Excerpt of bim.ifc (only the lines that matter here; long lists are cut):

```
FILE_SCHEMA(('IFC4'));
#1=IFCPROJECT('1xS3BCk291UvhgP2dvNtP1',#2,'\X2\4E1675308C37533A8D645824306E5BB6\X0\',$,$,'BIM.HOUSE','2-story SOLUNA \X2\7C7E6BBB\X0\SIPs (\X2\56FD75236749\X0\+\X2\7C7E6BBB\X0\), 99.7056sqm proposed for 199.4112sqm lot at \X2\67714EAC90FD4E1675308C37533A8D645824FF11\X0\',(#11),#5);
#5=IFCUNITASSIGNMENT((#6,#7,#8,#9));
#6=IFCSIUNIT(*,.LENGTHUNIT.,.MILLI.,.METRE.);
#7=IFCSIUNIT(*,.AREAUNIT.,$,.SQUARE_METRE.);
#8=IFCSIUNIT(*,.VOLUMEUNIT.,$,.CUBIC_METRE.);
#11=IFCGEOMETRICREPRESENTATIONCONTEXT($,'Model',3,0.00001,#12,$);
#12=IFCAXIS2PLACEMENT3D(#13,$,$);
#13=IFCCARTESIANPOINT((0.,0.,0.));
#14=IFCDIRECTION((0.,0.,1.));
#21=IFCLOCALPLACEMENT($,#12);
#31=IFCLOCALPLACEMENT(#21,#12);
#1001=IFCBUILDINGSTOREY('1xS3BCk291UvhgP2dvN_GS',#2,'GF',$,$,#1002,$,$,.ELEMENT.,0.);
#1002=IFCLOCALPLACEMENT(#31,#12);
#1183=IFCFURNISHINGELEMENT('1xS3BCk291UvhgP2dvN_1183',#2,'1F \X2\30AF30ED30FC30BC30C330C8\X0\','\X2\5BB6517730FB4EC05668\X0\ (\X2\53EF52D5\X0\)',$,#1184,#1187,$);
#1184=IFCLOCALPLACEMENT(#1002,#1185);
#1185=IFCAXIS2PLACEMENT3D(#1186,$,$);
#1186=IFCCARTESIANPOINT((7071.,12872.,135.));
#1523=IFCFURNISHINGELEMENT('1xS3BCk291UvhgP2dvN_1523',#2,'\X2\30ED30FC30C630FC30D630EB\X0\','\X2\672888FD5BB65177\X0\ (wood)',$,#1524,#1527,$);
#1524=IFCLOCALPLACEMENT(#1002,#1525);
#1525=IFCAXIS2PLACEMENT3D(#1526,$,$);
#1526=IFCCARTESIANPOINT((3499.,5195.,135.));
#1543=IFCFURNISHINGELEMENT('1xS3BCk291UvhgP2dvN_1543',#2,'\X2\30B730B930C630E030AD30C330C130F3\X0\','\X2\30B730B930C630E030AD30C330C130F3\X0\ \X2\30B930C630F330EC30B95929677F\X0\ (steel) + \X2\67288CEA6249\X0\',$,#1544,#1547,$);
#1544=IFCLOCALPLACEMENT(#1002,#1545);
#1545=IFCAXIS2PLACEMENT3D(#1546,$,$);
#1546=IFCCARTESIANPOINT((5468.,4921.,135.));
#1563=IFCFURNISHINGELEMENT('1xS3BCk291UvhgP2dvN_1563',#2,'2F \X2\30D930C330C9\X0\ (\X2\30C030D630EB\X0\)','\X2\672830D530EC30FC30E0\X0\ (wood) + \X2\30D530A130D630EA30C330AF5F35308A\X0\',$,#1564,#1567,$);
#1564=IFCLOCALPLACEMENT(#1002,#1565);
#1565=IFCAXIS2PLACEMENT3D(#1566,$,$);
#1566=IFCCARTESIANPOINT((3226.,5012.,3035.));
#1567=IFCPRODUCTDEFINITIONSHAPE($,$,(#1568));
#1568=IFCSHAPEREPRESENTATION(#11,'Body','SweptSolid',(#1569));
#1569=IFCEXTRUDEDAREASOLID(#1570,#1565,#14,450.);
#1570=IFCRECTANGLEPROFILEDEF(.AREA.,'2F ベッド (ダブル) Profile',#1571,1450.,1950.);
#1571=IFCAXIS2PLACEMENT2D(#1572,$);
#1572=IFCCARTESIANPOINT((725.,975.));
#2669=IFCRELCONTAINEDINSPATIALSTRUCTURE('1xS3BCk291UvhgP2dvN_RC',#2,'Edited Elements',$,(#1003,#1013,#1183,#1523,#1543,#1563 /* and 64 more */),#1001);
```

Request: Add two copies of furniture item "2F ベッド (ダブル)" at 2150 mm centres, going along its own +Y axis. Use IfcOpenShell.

```python
import ifcopenshell
import ifcopenshell.api.geometry
import ifcopenshell.api.root
import ifcopenshell.util.element
import ifcopenshell.util.placement
import ifcopenshell.util.unit

model = ifcopenshell.open("bim.ifc")
unit_scale = ifcopenshell.util.unit.calculate_unit_scale(model)


def reuse_history(source, copy):
    """copy_class also copies each property set's owner history, people and application; keep the originals."""
    for rel in copy.IsDefinedBy:
        if rel.is_a("IfcRelDefinesByProperties") and (history := rel.RelatingPropertyDefinition.OwnerHistory):
            rel.RelatingPropertyDefinition.OwnerHistory = source.OwnerHistory
            ifcopenshell.util.element.remove_deep2(model, history)


source = model.by_id(1563)
base = ifcopenshell.util.placement.get_local_placement(source.ObjectPlacement)
step = base[:3, 1] * 2.15 / unit_scale

for i in range(1, 3):
    copy = ifcopenshell.api.root.copy_class(model, product=source)
    copy.Representation = ifcopenshell.util.element.copy_deep(
        model, source.Representation, exclude=["IfcGeometricRepresentationContext", "IfcRepresentationMap"]
    )
    reuse_history(source, copy)
    matrix = base.copy()
    matrix[:3, 3] += i * step
    print("added at", matrix[:3, 3].round(3) + 0.0)
    ifcopenshell.api.geometry.edit_object_placement(model, product=copy, matrix=matrix, is_si=False)

model.write("bim_v2.ifc")
```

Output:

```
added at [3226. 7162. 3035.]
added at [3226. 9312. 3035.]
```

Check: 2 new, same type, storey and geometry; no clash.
